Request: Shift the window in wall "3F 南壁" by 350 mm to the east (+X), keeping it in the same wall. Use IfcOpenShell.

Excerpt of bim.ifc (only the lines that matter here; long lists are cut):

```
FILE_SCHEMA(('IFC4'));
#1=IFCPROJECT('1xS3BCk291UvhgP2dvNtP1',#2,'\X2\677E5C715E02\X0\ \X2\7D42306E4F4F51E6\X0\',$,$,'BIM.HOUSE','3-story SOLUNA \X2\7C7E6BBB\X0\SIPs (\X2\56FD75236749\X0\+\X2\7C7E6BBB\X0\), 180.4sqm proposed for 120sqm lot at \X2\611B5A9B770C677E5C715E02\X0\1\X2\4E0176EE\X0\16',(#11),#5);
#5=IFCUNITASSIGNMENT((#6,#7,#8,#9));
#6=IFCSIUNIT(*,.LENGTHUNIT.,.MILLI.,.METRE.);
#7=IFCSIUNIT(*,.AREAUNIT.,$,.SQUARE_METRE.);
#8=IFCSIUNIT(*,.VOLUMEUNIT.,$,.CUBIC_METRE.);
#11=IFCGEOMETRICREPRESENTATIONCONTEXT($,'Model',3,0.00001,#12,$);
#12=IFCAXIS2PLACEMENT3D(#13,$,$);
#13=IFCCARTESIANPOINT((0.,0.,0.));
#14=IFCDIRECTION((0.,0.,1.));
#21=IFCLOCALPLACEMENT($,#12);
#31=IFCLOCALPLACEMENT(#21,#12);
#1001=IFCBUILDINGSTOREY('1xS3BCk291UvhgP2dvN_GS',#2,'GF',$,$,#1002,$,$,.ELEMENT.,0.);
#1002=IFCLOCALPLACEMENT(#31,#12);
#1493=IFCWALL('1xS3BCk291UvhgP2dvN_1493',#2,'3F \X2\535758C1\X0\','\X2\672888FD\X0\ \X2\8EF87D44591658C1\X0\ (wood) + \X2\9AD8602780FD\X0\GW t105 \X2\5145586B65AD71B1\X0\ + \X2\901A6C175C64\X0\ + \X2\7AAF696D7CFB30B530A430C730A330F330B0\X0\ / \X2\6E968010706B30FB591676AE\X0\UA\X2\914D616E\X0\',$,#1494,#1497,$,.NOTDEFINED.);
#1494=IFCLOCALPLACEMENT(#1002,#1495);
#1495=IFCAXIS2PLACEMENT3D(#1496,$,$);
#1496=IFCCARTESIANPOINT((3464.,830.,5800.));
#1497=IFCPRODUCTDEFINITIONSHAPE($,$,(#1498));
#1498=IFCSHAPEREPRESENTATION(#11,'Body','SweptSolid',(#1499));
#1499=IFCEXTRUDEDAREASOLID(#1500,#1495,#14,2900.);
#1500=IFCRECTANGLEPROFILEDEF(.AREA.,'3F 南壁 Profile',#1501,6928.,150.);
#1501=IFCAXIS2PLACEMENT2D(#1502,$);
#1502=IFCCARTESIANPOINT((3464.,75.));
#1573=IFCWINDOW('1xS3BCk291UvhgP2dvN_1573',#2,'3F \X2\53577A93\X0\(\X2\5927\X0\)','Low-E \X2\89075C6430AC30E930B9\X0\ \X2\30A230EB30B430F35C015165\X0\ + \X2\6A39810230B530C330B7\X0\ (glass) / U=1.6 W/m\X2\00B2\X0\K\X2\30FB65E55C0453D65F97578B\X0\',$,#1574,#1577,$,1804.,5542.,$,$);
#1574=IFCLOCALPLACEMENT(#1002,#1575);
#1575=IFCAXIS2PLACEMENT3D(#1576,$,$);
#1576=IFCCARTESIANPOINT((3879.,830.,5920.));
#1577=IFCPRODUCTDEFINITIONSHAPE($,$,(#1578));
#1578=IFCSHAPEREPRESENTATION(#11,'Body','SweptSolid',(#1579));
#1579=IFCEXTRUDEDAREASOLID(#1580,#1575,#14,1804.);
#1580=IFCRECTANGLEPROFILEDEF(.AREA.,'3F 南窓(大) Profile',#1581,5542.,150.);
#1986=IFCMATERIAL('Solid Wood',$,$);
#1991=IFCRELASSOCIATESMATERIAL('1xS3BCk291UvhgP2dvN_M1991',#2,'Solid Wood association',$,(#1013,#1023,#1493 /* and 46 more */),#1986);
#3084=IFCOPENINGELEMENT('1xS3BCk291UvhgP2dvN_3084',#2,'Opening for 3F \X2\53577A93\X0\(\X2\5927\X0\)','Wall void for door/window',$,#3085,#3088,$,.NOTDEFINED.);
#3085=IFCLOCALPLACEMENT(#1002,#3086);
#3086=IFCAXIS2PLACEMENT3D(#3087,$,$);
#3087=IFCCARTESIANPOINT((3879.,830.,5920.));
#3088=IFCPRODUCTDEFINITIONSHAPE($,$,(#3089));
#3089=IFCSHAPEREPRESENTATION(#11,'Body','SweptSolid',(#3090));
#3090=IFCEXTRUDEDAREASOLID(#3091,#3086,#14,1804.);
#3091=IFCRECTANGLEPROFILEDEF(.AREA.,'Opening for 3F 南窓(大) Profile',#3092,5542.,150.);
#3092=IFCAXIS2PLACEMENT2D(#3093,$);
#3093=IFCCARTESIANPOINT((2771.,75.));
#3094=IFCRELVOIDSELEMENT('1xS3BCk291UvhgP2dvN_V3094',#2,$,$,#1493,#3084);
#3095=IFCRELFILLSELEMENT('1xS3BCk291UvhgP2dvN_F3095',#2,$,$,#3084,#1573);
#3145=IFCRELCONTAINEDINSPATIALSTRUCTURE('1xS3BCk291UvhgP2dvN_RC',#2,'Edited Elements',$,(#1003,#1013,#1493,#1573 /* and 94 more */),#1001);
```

```python
import ifcopenshell
import ifcopenshell.api.geometry
import ifcopenshell.util.placement
import ifcopenshell.util.unit

model = ifcopenshell.open("bim.ifc")
unit_scale = ifcopenshell.util.unit.calculate_unit_scale(model)

window = model.by_id(1573)
opening = window.FillsVoids[0].RelatingOpeningElement
wall = opening.VoidsElements[0].RelatingBuildingElement

wall_matrix = ifcopenshell.util.placement.get_local_placement(wall.ObjectPlacement)
shift = wall_matrix[:3, 0] * 0.35 / unit_scale
before = ifcopenshell.util.placement.get_local_placement(window.ObjectPlacement)[:3, 3].copy()

# The window is not placed relative to its opening, so move both.
for product in (opening, window):
    matrix = ifcopenshell.util.placement.get_local_placement(product.ObjectPlacement)
    matrix[:3, 3] += shift
    ifcopenshell.api.geometry.edit_object_placement(model, product=product, matrix=matrix, is_si=False)

after = ifcopenshell.util.placement.get_local_placement(window.ObjectPlacement)[:3, 3]
print("window moved by", (after - before).round(3) + 0.0)

model.write("bim_v2.ifc")
```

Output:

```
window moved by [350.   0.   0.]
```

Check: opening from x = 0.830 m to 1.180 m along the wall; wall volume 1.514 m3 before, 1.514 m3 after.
